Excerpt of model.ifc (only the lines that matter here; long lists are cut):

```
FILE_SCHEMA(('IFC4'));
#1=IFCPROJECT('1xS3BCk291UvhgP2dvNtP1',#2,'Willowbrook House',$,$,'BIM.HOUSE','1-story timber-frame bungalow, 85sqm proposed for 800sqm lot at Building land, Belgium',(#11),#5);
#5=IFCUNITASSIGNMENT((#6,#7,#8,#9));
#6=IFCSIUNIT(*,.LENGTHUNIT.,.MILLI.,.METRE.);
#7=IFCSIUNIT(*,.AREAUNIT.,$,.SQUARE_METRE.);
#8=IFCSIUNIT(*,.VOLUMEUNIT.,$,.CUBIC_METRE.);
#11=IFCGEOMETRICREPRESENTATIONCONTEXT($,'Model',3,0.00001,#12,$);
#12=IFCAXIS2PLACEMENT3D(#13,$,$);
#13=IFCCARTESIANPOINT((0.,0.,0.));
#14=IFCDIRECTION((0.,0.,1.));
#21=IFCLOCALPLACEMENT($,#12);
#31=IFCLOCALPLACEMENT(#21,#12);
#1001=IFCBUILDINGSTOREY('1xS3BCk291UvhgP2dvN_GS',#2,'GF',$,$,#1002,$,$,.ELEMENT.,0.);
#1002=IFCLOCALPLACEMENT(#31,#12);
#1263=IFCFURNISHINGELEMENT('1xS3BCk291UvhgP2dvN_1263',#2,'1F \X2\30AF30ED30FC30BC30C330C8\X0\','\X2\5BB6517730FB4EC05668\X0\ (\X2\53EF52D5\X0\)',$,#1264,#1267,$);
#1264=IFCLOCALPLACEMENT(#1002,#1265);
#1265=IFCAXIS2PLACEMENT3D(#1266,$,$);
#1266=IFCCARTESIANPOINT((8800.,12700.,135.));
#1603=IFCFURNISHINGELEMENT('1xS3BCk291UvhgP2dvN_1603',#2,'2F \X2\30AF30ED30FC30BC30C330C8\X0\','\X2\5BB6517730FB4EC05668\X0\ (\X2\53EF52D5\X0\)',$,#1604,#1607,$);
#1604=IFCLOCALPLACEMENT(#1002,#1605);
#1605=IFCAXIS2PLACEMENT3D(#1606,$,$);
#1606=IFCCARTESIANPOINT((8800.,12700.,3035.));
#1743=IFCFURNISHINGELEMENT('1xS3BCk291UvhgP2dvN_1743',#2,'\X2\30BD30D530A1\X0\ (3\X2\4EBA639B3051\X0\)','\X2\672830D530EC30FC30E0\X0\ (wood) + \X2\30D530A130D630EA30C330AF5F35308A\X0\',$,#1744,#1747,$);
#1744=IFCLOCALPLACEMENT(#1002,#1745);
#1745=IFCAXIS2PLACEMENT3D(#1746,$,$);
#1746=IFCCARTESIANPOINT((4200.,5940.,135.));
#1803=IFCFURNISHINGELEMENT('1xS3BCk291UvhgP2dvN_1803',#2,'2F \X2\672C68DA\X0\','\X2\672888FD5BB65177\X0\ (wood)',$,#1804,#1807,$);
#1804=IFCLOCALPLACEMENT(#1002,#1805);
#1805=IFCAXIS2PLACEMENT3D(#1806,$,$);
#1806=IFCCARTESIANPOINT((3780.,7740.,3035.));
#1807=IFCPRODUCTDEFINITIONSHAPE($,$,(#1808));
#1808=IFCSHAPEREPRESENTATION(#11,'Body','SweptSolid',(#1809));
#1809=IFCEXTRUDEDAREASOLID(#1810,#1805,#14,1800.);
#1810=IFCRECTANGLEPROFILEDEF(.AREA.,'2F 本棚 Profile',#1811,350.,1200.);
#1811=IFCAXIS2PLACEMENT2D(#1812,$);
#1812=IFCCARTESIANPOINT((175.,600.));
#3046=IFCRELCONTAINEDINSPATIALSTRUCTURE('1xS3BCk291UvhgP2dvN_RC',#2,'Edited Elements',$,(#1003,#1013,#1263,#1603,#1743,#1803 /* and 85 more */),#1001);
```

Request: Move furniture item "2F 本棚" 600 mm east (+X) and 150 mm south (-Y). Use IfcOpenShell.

```python
import ifcopenshell
import ifcopenshell.api.geometry
import ifcopenshell.util.placement
import ifcopenshell.util.unit

model = ifcopenshell.open("model.ifc")
unit_scale = ifcopenshell.util.unit.calculate_unit_scale(model)

item = model.by_id(1803)
matrix = ifcopenshell.util.placement.get_local_placement(item.ObjectPlacement)
matrix[0, 3] += 0.6 / unit_scale
matrix[1, 3] -= 0.15 / unit_scale
ifcopenshell.api.geometry.edit_object_placement(model, product=item, matrix=matrix, is_si=False)

print(ifcopenshell.util.placement.get_local_placement(item.ObjectPlacement).round(3) + 0.0)

model.write("model_rev.ifc")
```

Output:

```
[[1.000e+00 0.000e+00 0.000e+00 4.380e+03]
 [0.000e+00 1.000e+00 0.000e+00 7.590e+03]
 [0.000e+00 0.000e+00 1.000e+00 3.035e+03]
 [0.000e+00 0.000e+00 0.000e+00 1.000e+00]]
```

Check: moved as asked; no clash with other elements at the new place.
